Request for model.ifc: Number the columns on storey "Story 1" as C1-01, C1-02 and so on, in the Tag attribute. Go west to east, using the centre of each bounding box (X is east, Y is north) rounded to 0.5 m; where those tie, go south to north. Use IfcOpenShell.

First a look at what the model holds.

```python
import ifcopenshell
import ifcopenshell.util.element
import ifcopenshell.util.placement

model = ifcopenshell.open("model.ifc")
print(model.schema)
storey = next(s for s in model.by_type("IfcBuildingStorey") if s.Name == "Story 1")
columns = [e for e in ifcopenshell.util.element.get_decomposition(storey) if e.is_a("IfcColumn")]
for e in sorted(columns, key=lambda e: e.id()):
    origin = ifcopenshell.util.placement.get_local_placement(e.ObjectPlacement)[:3, 3]
    print(e.id(), e.Tag, e.Name, origin.round(2) + 0.0, sep=" | ")
```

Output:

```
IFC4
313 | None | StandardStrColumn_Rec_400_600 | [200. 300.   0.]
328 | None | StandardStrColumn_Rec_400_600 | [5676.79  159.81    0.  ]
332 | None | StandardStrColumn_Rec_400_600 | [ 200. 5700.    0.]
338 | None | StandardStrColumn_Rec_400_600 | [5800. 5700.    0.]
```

```python
import ifcopenshell
import ifcopenshell.geom
import ifcopenshell.util.element
import ifcopenshell.util.shape

model = ifcopenshell.open("model.ifc")
settings = ifcopenshell.geom.settings()
settings.set("use-world-coords", True)


def centre(element):
    shape = ifcopenshell.geom.create_shape(settings, element)
    return ifcopenshell.util.shape.get_bbox_centroid(shape.geometry)


storey = next(s for s in model.by_type("IfcBuildingStorey") if s.Name == "Story 1")
columns = [e for e in ifcopenshell.util.element.get_decomposition(storey) if e.is_a("IfcColumn")]

# Insertion points can sit at a corner or the storey origin, so sort by the geometry (in metres).
centres = {e: centre(e) for e in columns}
columns.sort(key=lambda e: (round(centres[e][0] / 0.5), centres[e][1]))

for i, e in enumerate(columns, start=1):
    number = f"C1-{i:02d}"
    e.Tag = number
    print(e.id(), number)

model.write("model_v2.ifc")
```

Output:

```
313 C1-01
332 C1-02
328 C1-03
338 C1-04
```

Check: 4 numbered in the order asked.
